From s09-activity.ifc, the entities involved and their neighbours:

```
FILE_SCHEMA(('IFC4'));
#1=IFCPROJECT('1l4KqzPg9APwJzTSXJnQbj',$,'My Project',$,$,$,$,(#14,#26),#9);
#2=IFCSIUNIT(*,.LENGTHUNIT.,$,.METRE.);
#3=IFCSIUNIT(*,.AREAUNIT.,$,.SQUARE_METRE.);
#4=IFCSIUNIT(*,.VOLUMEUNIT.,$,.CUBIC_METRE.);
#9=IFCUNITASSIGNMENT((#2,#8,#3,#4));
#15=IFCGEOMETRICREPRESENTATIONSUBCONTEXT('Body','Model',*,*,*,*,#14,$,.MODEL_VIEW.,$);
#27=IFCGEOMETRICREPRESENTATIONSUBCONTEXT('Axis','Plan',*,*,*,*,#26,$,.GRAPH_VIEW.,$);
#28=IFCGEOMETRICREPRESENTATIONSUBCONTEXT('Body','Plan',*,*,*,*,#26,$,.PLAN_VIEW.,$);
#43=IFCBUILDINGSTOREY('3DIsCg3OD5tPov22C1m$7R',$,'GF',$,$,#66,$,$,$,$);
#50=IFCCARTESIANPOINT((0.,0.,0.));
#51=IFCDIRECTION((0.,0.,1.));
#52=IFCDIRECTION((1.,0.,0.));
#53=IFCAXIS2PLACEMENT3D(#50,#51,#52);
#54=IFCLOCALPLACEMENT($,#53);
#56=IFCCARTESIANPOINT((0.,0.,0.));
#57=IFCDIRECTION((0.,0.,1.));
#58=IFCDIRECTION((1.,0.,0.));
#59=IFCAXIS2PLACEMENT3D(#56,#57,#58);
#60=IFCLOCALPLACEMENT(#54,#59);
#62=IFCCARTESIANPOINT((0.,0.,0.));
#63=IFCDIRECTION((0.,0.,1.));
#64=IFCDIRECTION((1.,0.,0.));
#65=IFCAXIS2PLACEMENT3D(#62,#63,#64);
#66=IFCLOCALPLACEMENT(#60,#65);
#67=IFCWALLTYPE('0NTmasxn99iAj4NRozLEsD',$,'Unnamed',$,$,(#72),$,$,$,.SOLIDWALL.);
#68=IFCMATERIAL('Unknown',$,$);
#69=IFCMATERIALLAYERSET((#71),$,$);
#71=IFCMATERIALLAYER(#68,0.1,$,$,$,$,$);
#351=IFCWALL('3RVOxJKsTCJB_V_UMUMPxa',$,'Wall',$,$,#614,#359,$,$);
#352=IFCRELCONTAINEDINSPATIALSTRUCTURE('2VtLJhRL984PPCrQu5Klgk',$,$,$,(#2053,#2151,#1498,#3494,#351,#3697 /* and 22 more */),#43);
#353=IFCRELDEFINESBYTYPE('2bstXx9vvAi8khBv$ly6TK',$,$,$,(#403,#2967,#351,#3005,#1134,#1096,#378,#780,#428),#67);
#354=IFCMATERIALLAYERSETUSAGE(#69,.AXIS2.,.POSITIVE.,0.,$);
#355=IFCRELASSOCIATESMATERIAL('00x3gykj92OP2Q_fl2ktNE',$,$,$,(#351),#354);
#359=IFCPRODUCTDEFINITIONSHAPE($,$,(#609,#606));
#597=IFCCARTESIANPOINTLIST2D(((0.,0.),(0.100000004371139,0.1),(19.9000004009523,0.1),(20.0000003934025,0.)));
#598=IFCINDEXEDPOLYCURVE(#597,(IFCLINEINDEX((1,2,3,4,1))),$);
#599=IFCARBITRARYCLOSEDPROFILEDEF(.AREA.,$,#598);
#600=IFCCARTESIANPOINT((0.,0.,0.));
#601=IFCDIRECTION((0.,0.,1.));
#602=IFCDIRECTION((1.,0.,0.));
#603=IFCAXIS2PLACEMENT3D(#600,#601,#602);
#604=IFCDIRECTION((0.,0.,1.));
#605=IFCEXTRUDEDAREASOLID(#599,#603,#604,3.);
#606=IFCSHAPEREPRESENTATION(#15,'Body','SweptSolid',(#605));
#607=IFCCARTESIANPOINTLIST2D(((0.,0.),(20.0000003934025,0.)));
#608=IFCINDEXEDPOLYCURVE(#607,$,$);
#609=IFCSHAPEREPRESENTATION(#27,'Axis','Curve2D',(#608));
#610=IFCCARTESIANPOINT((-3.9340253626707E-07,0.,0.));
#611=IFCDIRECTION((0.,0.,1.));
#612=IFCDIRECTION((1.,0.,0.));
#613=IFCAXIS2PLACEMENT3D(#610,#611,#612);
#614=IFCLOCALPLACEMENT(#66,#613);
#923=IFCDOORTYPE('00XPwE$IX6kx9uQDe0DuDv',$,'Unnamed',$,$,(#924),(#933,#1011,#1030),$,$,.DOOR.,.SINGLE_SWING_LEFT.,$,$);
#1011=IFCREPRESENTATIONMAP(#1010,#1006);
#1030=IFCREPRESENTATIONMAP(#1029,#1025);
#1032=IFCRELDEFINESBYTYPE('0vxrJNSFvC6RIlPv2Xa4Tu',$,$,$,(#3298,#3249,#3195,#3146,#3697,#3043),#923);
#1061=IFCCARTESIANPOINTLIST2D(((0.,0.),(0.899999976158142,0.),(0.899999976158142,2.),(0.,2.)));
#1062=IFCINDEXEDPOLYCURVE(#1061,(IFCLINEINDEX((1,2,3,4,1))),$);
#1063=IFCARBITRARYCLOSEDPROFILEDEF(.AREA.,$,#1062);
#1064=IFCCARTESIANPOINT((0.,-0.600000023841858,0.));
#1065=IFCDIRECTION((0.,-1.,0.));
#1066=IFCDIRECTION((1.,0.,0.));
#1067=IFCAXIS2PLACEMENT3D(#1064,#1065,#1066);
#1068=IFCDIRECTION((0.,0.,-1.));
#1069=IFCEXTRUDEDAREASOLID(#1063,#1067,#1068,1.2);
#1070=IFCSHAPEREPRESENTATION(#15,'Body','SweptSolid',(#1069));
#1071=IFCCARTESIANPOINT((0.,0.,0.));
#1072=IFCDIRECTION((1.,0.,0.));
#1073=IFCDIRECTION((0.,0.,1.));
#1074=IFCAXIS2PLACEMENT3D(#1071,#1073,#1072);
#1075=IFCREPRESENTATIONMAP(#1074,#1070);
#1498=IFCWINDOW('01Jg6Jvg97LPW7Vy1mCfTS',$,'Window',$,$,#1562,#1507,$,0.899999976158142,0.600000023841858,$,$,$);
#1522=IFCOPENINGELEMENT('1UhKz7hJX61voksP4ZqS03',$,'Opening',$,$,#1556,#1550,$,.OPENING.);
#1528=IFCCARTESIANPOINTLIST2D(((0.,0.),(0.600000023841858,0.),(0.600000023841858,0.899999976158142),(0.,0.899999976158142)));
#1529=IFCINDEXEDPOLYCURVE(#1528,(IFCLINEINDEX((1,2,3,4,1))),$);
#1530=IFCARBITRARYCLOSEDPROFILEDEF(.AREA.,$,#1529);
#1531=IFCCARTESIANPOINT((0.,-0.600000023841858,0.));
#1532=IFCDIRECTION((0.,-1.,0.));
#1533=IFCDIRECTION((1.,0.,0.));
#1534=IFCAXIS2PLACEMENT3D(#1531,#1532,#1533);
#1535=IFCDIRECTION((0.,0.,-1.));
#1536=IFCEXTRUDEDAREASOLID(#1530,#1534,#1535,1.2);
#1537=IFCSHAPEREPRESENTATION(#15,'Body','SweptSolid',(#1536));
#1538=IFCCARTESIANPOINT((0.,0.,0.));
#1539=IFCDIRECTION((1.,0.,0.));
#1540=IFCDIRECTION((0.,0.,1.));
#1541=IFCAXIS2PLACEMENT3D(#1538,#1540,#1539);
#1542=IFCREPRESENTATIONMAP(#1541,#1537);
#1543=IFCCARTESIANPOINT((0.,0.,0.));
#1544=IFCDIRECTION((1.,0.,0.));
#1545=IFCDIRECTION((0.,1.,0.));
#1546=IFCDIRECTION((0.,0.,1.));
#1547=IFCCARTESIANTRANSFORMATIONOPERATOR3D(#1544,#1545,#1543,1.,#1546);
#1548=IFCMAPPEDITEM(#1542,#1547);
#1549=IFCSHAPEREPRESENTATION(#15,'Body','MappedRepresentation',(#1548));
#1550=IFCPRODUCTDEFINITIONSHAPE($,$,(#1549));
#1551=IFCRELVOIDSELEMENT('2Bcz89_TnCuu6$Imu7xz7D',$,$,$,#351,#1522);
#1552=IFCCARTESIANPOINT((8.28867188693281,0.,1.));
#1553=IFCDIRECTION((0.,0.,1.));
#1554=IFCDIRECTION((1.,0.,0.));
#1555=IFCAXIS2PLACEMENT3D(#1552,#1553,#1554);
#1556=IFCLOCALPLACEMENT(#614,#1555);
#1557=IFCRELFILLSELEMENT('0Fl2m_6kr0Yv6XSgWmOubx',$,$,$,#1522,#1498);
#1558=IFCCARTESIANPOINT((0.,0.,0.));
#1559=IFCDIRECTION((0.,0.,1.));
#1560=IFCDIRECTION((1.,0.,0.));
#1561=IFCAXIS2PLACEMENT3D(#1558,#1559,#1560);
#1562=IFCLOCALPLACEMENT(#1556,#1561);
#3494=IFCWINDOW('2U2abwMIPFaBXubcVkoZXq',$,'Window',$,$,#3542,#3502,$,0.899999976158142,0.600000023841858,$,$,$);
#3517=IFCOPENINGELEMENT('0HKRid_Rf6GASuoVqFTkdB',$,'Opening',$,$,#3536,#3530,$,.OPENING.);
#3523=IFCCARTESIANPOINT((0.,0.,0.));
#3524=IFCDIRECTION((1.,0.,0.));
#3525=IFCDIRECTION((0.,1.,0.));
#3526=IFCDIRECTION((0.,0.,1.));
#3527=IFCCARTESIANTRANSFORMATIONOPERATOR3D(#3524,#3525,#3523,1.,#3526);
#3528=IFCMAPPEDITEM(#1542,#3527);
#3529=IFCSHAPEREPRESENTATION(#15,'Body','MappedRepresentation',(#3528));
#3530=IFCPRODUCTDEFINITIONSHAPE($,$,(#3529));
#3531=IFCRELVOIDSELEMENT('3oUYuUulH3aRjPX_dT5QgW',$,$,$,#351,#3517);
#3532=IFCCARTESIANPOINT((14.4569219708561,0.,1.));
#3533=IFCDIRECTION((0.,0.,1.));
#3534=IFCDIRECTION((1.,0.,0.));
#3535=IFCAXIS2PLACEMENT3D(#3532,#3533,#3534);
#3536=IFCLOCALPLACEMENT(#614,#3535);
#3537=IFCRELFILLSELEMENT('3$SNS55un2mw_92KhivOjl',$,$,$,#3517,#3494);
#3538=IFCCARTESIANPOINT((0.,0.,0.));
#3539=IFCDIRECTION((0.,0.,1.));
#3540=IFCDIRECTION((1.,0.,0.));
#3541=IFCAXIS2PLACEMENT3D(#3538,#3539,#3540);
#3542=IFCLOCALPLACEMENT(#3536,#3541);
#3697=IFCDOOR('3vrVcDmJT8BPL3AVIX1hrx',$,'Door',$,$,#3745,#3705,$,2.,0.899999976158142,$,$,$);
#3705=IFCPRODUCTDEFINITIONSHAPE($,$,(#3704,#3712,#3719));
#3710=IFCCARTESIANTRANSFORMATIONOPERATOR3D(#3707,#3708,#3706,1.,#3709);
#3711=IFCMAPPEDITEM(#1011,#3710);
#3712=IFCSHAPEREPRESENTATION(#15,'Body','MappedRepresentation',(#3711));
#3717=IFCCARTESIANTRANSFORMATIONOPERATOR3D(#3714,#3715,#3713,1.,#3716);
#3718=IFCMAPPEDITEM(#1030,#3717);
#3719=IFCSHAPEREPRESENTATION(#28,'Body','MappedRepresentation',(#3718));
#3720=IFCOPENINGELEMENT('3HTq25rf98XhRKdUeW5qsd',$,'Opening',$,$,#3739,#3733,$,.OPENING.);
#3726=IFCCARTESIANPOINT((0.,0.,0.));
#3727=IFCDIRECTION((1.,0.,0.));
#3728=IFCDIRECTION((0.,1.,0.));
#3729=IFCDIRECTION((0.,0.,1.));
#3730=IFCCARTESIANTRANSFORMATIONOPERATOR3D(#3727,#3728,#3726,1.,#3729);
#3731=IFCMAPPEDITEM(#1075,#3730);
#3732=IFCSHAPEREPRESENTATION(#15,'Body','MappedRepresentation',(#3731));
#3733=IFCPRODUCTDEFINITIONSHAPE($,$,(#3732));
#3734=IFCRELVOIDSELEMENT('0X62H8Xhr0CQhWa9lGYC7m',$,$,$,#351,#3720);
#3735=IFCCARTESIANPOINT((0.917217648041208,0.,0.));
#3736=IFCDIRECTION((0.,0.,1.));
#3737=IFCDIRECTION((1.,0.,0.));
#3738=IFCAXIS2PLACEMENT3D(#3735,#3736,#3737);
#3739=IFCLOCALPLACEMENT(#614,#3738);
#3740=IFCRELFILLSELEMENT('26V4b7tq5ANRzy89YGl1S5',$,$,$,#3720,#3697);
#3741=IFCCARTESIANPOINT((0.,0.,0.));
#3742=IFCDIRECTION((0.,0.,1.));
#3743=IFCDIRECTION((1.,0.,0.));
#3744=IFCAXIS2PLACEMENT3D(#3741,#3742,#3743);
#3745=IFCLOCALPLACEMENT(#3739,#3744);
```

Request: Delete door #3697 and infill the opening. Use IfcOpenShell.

```python
import ifcopenshell
import ifcopenshell.api.feature
import ifcopenshell.api.root
import ifcopenshell.geom
import ifcopenshell.util.shape

model = ifcopenshell.open("s09-activity.ifc")
settings = ifcopenshell.geom.settings()


def volume(element):
    """Net volume in cubic metres, openings subtracted."""
    shape = ifcopenshell.geom.create_shape(settings, element)
    return ifcopenshell.util.shape.get_volume(shape.geometry)


door = model.by_guid("3vrVcDmJT8BPL3AVIX1hrx")
opening = door.FillsVoids[0].RelatingOpeningElement
wall = opening.VoidsElements[0].RelatingBuildingElement
before = volume(wall)

ifcopenshell.api.root.remove_product(model, product=door)
ifcopenshell.api.feature.remove_feature(model, feature=opening)

after = volume(wall)

print(f"wall volume {before:.3f} -> {after:.3f} m3")

model.write("s09-activity-out.ifc")
```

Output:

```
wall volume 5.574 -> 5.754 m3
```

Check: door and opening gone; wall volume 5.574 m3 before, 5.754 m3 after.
